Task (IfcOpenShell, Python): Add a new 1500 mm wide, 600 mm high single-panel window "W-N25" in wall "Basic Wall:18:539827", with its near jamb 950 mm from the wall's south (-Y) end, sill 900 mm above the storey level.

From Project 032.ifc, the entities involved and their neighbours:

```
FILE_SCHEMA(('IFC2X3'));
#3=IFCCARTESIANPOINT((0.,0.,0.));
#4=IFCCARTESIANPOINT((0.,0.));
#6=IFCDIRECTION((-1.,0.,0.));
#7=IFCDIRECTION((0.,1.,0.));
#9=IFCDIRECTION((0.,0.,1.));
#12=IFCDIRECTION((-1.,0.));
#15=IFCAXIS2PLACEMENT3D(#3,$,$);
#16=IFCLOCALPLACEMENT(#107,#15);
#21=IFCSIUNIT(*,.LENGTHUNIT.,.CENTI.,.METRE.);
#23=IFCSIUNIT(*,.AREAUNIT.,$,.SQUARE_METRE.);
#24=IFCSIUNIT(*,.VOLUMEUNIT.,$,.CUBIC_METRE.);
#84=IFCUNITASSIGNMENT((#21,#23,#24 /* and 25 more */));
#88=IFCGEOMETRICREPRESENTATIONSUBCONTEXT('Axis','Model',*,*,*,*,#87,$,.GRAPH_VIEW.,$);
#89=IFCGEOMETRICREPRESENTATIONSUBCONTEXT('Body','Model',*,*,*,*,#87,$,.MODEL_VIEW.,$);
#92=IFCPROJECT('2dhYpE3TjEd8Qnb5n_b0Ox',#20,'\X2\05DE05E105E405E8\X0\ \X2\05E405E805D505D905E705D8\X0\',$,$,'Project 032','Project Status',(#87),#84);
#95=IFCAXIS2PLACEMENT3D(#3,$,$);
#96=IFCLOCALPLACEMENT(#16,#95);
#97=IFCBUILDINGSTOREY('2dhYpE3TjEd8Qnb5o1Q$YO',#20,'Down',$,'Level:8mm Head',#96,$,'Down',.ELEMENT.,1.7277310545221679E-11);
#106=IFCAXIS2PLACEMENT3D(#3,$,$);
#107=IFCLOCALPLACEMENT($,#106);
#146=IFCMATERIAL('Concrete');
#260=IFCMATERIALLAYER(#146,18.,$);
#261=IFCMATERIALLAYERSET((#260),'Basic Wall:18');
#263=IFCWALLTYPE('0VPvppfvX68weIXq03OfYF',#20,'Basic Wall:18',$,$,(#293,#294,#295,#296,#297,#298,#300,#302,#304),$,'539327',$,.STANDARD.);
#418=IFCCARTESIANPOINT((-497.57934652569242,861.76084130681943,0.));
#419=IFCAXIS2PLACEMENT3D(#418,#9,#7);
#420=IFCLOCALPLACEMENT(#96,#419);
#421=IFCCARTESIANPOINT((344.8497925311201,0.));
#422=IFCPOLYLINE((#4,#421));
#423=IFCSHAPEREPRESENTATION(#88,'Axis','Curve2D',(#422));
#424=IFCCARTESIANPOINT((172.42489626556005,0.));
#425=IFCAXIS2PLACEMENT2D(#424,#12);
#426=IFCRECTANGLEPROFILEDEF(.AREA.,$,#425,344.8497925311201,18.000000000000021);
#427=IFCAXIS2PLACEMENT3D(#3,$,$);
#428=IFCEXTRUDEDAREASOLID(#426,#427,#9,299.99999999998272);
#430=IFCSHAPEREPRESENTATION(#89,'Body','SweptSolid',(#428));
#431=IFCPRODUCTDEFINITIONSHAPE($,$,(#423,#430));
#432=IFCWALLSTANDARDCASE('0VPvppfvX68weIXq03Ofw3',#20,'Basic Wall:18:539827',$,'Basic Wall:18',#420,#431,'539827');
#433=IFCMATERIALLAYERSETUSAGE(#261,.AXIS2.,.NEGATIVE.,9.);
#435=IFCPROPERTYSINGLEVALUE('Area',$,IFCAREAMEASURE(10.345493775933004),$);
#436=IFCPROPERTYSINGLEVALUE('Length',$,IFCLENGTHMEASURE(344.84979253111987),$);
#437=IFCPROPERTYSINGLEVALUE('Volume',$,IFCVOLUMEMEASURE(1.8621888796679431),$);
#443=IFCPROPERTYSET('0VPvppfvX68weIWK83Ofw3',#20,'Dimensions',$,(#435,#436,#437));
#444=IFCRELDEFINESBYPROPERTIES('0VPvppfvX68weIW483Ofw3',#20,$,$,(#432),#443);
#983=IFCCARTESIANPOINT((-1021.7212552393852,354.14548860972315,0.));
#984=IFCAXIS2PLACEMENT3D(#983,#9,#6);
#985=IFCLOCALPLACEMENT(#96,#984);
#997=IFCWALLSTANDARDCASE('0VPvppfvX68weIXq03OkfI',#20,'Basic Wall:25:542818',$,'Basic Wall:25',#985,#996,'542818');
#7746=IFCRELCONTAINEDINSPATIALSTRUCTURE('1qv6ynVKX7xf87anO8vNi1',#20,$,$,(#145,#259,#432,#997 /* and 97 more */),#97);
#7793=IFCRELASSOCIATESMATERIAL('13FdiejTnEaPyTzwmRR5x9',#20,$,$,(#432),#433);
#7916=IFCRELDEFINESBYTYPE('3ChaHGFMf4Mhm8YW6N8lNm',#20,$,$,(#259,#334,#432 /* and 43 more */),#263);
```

```python
import numpy as np
import ifcopenshell
import ifcopenshell.api.feature
import ifcopenshell.api.geometry
import ifcopenshell.api.pset
import ifcopenshell.api.root
import ifcopenshell.api.spatial
import ifcopenshell.api.type
import ifcopenshell.geom
import ifcopenshell.util.element
import ifcopenshell.util.placement
import ifcopenshell.util.representation
import ifcopenshell.util.shape
import ifcopenshell.util.unit

model = ifcopenshell.open("Project 032.ifc")
unit_scale = ifcopenshell.util.unit.calculate_unit_scale(model)
area_scale = ifcopenshell.util.unit.calculate_unit_scale(model, "AREAUNIT")
volume_scale = ifcopenshell.util.unit.calculate_unit_scale(model, "VOLUMEUNIT")
settings = ifcopenshell.geom.settings()


def volume(element):
    """Net volume in cubic metres, openings subtracted."""
    shape = ifcopenshell.geom.create_shape(settings, element)
    return ifcopenshell.util.shape.get_volume(shape.geometry)


wall = model.by_guid("0VPvppfvX68weIXq03Ofw3")
storey = ifcopenshell.util.element.get_container(wall, ifc_class="IfcBuildingStorey")
context = ifcopenshell.util.representation.get_context(model, "Model", "Body", "MODEL_VIEW")
before = volume(wall)

width, height, from_end, sill = 1.5, 0.6, 0.95, 0.9  # metres

# The wall runs along its own X axis, and the end named is its -X end.
wall_shape = ifcopenshell.geom.create_shape(settings, wall)
x, y, z = ifcopenshell.util.shape.get_vertices(wall_shape.geometry).T
start = x.min() + from_end
face, thickness = float(y.min()), float(y.max() - y.min())
wall_matrix = ifcopenshell.util.placement.get_local_placement(wall.ObjectPlacement)
level = ifcopenshell.util.placement.get_local_placement(storey.ObjectPlacement)[2, 3]


def in_wall(x, y):
    """Placement at x, y metres in the wall's axes, at sill height."""
    matrix = wall_matrix.copy()
    matrix[:, 3] = wall_matrix @ np.array([x / unit_scale, y / unit_scale, 0.0, 1.0])
    matrix[2, 3] = level + sill / unit_scale
    return matrix


# Opening: a box that overshoots both wall faces by 50 mm.
opening = ifcopenshell.api.root.create_entity(model, ifc_class="IfcOpeningElement")
box = ifcopenshell.api.geometry.add_wall_representation(
    model, context=context, length=width, height=height, thickness=thickness + 0.1
)
ifcopenshell.api.geometry.assign_representation(model, product=opening, representation=box)
ifcopenshell.api.geometry.edit_object_placement(model, product=opening, matrix=in_wall(start, face - 0.05), is_si=False)
ifcopenshell.api.feature.add_feature(model, feature=opening, element=wall)

window = ifcopenshell.api.root.create_entity(model, ifc_class="IfcWindow", name="W-N25")
window.OverallWidth, window.OverallHeight = width / unit_scale, height / unit_scale
body = ifcopenshell.api.geometry.add_window_representation(
    model,
    context=context,
    overall_width=window.OverallWidth,
    overall_height=window.OverallHeight,
    partition_type="SINGLE_PANEL",
)
ifcopenshell.api.geometry.assign_representation(model, product=window, representation=body)
ifcopenshell.api.spatial.assign_container(model, products=[window], relating_structure=storey)
fills = ifcopenshell.api.feature.add_filling(model, opening=opening, element=window)
fills.OwnerHistory = window.OwnerHistory  # required in IFC2X3

# IFC2X3 keeps the operation on the window style.
style = ifcopenshell.api.root.create_entity(model, ifc_class="IfcWindowStyle", name="W-N25")
style.OperationType, style.ConstructionType = "SINGLE_PANEL", "NOTDEFINED"
style.ParameterTakesPrecedence = style.Sizeable = False
ifcopenshell.api.type.assign_type(model, related_objects=[window], relating_type=style)

# Centre the window in the wall's thickness.
ifcopenshell.api.geometry.edit_object_placement(model, product=window, matrix=in_wall(start, face), is_si=False)
window_shape = ifcopenshell.geom.create_shape(settings, window)
depth = ifcopenshell.util.shape.get_vertices(window_shape.geometry)[:, 1]
offset = face + thickness / 2 - (depth.min() + depth.max()) / 2
ifcopenshell.api.geometry.edit_object_placement(model, product=window, matrix=in_wall(start, offset), is_si=False)

after = volume(wall)

# Update the wall's stored quantities.
pset = model.by_id(ifcopenshell.util.element.get_pset(wall, "Dimensions", should_inherit=False)["id"])
ifcopenshell.api.pset.edit_pset(model, pset=pset, properties={
    "Area": model.create_entity("IfcAreaMeasure", after / thickness / area_scale),
    "Volume": model.create_entity("IfcVolumeMeasure", after / volume_scale),
})

print(f"wall volume {before:.3f} -> {after:.3f} m3")

model.write("Project 032_edited.ifc")
```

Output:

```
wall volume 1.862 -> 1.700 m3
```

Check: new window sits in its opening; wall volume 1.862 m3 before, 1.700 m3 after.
